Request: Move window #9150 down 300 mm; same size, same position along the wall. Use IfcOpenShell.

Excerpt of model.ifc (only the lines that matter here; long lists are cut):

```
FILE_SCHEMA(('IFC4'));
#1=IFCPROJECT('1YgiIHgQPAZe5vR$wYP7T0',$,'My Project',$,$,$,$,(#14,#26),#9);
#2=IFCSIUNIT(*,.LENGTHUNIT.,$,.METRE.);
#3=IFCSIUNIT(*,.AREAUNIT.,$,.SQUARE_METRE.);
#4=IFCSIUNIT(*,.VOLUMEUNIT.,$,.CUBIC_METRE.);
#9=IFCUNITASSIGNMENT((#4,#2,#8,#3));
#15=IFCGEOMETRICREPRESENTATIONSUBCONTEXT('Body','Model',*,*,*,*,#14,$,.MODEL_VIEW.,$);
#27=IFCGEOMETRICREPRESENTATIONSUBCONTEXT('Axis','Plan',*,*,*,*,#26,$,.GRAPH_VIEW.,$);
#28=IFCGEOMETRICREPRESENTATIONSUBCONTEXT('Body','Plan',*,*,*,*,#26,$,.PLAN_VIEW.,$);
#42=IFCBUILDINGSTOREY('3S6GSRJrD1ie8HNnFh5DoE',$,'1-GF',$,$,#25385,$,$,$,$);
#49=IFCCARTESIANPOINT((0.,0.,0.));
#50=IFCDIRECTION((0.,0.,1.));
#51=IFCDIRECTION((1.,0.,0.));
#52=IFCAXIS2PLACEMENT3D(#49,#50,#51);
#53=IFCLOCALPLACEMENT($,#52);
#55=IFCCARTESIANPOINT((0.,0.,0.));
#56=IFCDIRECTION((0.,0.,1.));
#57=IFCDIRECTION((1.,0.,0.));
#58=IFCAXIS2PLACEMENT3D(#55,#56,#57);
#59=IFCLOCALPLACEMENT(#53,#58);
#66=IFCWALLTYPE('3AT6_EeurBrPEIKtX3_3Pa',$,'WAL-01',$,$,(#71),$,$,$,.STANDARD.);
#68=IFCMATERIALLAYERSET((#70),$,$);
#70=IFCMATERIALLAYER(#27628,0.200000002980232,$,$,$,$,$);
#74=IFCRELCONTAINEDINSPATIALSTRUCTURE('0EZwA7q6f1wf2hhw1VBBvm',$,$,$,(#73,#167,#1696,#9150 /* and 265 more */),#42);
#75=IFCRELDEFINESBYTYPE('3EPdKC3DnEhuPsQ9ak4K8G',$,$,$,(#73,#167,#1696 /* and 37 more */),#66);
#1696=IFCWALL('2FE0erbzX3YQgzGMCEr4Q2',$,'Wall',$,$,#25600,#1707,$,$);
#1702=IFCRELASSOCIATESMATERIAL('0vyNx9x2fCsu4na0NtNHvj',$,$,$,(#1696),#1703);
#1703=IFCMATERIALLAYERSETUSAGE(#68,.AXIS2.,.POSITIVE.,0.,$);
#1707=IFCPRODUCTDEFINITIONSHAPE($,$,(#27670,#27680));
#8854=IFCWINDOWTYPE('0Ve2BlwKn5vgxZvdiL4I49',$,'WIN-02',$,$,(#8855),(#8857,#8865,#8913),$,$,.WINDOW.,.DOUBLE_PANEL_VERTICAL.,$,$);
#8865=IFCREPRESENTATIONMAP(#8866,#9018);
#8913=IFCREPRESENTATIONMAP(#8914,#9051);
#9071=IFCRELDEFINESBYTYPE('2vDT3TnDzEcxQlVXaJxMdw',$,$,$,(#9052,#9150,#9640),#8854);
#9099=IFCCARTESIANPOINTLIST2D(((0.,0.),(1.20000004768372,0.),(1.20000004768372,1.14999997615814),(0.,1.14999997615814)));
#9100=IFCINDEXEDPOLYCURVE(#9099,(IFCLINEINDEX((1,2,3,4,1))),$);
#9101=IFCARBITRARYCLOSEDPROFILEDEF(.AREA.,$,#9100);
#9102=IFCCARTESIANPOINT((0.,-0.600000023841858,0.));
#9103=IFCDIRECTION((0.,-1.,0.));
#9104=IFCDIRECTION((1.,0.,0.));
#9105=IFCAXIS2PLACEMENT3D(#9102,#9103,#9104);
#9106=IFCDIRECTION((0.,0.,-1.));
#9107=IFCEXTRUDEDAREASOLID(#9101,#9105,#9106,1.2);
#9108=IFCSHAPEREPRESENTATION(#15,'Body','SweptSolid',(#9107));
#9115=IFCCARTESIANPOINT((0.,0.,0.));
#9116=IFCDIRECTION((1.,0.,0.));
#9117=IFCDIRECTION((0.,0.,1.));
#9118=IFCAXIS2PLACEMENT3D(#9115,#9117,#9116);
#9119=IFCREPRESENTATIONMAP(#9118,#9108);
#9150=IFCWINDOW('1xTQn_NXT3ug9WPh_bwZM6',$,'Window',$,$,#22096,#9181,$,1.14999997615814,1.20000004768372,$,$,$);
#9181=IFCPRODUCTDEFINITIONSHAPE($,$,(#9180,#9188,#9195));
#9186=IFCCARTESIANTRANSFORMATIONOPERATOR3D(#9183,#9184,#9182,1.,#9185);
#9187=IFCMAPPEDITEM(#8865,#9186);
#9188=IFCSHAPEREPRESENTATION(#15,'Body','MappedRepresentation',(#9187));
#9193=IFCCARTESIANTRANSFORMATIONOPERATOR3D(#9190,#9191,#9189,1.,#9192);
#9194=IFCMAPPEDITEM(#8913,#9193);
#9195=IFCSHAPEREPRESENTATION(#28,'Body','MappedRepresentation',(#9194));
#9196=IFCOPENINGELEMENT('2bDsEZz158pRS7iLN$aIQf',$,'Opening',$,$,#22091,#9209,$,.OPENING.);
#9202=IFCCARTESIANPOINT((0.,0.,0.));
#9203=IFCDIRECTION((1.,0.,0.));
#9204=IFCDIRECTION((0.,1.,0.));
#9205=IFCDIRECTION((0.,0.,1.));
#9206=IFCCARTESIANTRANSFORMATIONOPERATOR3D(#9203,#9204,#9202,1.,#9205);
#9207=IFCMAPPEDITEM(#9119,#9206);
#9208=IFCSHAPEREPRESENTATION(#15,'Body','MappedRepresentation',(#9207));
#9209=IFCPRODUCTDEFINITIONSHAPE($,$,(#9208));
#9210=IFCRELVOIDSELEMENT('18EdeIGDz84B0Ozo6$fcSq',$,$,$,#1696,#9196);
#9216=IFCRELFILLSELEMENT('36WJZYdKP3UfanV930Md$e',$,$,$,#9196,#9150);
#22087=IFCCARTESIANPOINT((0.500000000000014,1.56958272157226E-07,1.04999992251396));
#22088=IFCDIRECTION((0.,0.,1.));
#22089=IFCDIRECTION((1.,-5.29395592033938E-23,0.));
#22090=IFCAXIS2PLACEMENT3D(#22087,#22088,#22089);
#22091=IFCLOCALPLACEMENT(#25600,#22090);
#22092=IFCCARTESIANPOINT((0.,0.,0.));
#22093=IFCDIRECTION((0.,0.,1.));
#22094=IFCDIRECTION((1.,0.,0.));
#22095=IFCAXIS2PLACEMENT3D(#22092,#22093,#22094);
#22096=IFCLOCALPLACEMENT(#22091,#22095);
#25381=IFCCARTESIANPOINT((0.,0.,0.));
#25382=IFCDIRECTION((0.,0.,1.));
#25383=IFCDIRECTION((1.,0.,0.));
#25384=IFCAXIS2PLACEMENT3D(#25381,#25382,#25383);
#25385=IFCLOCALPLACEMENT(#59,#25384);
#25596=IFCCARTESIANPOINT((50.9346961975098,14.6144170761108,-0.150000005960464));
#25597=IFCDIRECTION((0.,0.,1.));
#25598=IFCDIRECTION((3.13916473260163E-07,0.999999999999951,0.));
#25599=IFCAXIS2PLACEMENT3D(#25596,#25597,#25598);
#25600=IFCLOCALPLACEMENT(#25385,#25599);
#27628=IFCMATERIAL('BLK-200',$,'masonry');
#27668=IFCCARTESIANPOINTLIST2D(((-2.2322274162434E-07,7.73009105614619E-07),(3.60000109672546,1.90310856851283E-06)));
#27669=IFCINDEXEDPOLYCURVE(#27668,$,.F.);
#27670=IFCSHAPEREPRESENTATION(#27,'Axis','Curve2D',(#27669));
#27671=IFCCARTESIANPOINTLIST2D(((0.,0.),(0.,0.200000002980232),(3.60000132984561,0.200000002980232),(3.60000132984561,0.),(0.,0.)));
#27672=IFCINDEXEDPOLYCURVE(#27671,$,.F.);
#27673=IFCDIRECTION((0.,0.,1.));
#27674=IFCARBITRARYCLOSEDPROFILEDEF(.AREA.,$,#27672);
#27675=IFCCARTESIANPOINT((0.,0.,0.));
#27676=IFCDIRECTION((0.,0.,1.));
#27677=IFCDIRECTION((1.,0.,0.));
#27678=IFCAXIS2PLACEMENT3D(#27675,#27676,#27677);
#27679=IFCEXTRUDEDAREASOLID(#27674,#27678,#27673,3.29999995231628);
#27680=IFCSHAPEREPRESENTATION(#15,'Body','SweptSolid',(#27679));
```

```python
import numpy as np
import ifcopenshell
import ifcopenshell.api.geometry
import ifcopenshell.util.placement
import ifcopenshell.util.unit

model = ifcopenshell.open("model.ifc")
unit_scale = ifcopenshell.util.unit.calculate_unit_scale(model)

window = model.by_guid("1xTQn_NXT3ug9WPh_bwZM6")
opening = window.FillsVoids[0].RelatingOpeningElement
dz = -0.3 / unit_scale

shift = np.array([0.0, 0.0, dz])
# The window is placed relative to its opening, so it follows when the opening moves.
matrix = ifcopenshell.util.placement.get_local_placement(opening.ObjectPlacement)
matrix[:3, 3] += shift
ifcopenshell.api.geometry.edit_object_placement(
    model, product=opening, matrix=matrix, is_si=False, should_transform_children=True
)

print(f"moved by {dz * unit_scale:+.3f} m")

model.write("model_v2.ifc")
```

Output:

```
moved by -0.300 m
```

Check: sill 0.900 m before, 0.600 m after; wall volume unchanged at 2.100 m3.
